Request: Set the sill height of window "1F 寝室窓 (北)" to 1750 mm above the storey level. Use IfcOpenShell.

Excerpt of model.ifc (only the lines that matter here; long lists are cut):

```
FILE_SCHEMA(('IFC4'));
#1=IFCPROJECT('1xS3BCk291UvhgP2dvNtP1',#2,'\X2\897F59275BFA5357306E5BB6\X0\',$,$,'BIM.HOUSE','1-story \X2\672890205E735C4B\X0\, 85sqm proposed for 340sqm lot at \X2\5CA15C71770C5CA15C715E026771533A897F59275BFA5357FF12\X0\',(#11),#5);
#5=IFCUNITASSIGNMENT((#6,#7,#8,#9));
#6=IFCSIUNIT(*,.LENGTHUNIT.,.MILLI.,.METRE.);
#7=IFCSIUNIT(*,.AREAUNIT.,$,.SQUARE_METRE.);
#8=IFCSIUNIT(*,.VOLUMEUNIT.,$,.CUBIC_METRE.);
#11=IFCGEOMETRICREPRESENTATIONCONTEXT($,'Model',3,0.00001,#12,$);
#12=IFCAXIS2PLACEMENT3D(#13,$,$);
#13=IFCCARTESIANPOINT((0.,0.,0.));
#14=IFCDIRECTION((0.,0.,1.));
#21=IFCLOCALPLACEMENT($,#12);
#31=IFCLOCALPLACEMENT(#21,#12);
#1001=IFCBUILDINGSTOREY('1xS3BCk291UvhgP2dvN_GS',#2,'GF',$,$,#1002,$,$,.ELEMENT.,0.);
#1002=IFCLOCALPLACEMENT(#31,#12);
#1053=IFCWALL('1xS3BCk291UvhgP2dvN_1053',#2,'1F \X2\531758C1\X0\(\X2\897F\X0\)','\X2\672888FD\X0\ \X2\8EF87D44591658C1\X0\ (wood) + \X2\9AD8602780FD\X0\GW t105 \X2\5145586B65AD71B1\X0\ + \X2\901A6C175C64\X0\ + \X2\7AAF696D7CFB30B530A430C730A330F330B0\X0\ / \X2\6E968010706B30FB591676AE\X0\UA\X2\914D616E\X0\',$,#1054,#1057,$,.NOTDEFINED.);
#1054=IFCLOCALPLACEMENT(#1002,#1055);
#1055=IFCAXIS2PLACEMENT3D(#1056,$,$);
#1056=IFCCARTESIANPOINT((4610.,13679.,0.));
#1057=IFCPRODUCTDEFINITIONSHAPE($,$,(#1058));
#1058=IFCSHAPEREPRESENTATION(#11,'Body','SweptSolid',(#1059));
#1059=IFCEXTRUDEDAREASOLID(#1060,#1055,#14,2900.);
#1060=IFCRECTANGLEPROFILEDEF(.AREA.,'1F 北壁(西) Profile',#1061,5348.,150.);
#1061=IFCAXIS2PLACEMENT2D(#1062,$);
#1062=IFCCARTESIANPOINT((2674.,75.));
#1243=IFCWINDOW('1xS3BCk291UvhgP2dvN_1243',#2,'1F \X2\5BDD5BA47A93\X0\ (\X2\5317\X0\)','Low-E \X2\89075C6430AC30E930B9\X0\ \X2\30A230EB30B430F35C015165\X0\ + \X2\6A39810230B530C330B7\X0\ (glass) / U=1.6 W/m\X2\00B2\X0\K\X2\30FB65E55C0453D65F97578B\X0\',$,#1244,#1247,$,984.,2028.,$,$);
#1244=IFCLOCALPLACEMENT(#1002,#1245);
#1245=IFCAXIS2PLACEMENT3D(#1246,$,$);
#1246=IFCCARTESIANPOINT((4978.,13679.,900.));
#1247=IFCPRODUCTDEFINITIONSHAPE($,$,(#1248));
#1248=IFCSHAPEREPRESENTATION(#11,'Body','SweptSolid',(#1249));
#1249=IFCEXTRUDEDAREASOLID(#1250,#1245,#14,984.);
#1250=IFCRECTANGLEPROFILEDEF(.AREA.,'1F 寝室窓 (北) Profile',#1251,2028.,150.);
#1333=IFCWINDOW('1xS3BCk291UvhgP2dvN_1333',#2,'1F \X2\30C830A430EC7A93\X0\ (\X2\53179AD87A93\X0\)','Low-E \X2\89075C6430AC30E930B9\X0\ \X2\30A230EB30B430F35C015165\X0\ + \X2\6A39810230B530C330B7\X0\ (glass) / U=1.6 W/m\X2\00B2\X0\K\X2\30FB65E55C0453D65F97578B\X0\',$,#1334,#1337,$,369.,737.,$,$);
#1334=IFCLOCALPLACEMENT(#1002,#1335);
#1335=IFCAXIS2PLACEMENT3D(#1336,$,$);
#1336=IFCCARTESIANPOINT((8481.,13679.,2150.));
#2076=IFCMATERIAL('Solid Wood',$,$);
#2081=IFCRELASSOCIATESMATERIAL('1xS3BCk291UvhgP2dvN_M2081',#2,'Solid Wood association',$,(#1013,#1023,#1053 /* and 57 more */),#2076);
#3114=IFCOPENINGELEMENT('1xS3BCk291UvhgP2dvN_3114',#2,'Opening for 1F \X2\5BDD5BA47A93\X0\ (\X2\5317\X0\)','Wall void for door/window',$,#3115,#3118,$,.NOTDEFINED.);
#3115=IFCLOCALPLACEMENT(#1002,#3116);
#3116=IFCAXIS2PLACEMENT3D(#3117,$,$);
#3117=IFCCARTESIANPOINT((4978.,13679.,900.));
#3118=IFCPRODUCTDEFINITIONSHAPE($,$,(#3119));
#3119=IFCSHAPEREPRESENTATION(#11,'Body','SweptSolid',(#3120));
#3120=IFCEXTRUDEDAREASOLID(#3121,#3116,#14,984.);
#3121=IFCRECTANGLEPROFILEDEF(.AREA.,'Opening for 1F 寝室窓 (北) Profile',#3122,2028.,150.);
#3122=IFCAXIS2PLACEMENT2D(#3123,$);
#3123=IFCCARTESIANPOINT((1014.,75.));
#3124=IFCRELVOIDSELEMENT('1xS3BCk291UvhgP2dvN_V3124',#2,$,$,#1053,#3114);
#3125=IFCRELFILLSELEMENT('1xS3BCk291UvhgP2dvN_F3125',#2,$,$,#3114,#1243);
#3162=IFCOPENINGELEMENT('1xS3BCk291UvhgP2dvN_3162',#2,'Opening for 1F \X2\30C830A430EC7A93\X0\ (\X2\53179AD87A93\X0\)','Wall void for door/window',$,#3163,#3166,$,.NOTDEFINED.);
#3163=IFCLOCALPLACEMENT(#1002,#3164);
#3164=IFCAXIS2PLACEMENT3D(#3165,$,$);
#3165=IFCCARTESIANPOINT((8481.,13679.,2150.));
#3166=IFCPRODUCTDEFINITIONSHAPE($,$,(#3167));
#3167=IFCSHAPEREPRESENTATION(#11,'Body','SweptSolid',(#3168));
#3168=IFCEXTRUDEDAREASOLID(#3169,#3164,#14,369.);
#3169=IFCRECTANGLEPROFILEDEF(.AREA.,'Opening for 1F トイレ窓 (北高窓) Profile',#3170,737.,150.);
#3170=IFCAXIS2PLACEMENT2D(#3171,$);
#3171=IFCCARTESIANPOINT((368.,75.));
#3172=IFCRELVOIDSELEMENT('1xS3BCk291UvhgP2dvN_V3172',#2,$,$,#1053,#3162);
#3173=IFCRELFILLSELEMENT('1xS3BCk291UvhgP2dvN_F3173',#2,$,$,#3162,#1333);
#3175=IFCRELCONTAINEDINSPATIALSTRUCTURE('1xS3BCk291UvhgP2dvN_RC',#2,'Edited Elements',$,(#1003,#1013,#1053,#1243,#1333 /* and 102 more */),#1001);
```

```python
import numpy as np
import ifcopenshell
import ifcopenshell.api.geometry
import ifcopenshell.geom
import ifcopenshell.util.element
import ifcopenshell.util.placement
import ifcopenshell.util.shape
import ifcopenshell.util.unit

model = ifcopenshell.open("model.ifc")
unit_scale = ifcopenshell.util.unit.calculate_unit_scale(model)

window = model.by_id(1243)
opening = window.FillsVoids[0].RelatingOpeningElement
storey = ifcopenshell.util.element.get_container(window, ifc_class="IfcBuildingStorey")
level = ifcopenshell.util.placement.get_local_placement(storey.ObjectPlacement)[2, 3]

# The opening's origin need not be at the sill, so measure its lowest point.
shape = ifcopenshell.geom.create_shape(ifcopenshell.geom.settings(), opening)
bottom = ifcopenshell.util.shape.get_shape_bottom_elevation(shape, shape.geometry) / unit_scale
dz = level + 1.75 / unit_scale - bottom

shift = np.array([0.0, 0.0, dz])
# The window is not placed relative to its opening, so move both.
for product in (opening, window):
    matrix = ifcopenshell.util.placement.get_local_placement(product.ObjectPlacement)
    matrix[:3, 3] += shift
    ifcopenshell.api.geometry.edit_object_placement(model, product=product, matrix=matrix, is_si=False)

print(f"moved by {dz * unit_scale:+.3f} m")

model.write("model-out.ifc")
```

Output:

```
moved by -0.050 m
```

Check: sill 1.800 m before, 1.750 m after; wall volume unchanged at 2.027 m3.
